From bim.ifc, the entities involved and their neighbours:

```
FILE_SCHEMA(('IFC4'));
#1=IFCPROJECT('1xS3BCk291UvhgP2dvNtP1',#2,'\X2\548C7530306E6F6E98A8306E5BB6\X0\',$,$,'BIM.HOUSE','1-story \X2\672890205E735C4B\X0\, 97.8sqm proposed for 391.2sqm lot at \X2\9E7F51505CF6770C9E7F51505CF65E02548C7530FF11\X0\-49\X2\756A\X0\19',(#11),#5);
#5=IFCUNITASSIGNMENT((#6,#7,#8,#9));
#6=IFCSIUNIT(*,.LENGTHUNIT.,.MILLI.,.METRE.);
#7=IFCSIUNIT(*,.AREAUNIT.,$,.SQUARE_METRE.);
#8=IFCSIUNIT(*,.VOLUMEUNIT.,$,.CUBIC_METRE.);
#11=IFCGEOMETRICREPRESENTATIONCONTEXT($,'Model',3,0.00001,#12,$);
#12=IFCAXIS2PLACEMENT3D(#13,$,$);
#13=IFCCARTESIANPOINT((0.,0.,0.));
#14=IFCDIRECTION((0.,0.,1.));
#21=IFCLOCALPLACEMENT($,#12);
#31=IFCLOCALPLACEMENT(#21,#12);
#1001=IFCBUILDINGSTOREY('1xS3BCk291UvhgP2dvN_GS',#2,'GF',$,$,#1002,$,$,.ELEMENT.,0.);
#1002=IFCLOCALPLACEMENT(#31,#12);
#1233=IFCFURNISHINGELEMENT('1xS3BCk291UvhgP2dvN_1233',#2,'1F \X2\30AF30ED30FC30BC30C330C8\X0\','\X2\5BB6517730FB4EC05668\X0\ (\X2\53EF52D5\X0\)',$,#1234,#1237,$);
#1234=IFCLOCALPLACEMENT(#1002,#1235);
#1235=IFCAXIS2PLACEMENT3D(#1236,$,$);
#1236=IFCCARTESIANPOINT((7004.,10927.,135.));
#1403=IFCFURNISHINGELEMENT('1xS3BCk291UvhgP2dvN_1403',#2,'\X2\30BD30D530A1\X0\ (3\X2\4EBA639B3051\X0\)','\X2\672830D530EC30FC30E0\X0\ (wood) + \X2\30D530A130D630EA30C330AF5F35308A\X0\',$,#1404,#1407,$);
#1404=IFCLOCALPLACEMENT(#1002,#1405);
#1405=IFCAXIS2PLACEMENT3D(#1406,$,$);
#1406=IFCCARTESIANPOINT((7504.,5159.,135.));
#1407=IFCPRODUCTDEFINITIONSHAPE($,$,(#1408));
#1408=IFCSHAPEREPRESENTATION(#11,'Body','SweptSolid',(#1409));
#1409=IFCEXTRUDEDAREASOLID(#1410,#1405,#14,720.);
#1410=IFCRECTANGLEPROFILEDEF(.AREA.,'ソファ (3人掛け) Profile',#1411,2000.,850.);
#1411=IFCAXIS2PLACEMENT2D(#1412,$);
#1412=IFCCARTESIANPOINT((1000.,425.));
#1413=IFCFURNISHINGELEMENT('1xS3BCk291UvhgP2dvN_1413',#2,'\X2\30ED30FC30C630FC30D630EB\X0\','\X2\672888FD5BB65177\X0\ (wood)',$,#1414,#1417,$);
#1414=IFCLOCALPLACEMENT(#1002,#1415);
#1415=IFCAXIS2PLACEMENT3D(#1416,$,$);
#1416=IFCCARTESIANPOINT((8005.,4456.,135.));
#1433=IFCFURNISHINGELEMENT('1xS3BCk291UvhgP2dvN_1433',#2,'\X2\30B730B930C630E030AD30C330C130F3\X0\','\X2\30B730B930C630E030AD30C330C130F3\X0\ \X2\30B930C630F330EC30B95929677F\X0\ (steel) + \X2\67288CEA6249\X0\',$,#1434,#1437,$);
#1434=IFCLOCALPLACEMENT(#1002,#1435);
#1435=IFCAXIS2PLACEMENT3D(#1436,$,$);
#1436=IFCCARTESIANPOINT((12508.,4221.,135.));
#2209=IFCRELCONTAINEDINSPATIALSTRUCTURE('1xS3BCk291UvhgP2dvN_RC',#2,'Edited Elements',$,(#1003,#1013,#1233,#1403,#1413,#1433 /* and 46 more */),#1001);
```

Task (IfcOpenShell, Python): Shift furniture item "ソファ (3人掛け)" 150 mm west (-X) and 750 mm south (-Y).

```python
import ifcopenshell
import ifcopenshell.api.geometry
import ifcopenshell.util.placement
import ifcopenshell.util.unit

model = ifcopenshell.open("bim.ifc")
unit_scale = ifcopenshell.util.unit.calculate_unit_scale(model)

item = model.by_id(1403)
matrix = ifcopenshell.util.placement.get_local_placement(item.ObjectPlacement)
matrix[0, 3] -= 0.15 / unit_scale
matrix[1, 3] -= 0.75 / unit_scale
ifcopenshell.api.geometry.edit_object_placement(model, product=item, matrix=matrix, is_si=False)

print(ifcopenshell.util.placement.get_local_placement(item.ObjectPlacement).round(3) + 0.0)

model.write("bim_rev.ifc")
```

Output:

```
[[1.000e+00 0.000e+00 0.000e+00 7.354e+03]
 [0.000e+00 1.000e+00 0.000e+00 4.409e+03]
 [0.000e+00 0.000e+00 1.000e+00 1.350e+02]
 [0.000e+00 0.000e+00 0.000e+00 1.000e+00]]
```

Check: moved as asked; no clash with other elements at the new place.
